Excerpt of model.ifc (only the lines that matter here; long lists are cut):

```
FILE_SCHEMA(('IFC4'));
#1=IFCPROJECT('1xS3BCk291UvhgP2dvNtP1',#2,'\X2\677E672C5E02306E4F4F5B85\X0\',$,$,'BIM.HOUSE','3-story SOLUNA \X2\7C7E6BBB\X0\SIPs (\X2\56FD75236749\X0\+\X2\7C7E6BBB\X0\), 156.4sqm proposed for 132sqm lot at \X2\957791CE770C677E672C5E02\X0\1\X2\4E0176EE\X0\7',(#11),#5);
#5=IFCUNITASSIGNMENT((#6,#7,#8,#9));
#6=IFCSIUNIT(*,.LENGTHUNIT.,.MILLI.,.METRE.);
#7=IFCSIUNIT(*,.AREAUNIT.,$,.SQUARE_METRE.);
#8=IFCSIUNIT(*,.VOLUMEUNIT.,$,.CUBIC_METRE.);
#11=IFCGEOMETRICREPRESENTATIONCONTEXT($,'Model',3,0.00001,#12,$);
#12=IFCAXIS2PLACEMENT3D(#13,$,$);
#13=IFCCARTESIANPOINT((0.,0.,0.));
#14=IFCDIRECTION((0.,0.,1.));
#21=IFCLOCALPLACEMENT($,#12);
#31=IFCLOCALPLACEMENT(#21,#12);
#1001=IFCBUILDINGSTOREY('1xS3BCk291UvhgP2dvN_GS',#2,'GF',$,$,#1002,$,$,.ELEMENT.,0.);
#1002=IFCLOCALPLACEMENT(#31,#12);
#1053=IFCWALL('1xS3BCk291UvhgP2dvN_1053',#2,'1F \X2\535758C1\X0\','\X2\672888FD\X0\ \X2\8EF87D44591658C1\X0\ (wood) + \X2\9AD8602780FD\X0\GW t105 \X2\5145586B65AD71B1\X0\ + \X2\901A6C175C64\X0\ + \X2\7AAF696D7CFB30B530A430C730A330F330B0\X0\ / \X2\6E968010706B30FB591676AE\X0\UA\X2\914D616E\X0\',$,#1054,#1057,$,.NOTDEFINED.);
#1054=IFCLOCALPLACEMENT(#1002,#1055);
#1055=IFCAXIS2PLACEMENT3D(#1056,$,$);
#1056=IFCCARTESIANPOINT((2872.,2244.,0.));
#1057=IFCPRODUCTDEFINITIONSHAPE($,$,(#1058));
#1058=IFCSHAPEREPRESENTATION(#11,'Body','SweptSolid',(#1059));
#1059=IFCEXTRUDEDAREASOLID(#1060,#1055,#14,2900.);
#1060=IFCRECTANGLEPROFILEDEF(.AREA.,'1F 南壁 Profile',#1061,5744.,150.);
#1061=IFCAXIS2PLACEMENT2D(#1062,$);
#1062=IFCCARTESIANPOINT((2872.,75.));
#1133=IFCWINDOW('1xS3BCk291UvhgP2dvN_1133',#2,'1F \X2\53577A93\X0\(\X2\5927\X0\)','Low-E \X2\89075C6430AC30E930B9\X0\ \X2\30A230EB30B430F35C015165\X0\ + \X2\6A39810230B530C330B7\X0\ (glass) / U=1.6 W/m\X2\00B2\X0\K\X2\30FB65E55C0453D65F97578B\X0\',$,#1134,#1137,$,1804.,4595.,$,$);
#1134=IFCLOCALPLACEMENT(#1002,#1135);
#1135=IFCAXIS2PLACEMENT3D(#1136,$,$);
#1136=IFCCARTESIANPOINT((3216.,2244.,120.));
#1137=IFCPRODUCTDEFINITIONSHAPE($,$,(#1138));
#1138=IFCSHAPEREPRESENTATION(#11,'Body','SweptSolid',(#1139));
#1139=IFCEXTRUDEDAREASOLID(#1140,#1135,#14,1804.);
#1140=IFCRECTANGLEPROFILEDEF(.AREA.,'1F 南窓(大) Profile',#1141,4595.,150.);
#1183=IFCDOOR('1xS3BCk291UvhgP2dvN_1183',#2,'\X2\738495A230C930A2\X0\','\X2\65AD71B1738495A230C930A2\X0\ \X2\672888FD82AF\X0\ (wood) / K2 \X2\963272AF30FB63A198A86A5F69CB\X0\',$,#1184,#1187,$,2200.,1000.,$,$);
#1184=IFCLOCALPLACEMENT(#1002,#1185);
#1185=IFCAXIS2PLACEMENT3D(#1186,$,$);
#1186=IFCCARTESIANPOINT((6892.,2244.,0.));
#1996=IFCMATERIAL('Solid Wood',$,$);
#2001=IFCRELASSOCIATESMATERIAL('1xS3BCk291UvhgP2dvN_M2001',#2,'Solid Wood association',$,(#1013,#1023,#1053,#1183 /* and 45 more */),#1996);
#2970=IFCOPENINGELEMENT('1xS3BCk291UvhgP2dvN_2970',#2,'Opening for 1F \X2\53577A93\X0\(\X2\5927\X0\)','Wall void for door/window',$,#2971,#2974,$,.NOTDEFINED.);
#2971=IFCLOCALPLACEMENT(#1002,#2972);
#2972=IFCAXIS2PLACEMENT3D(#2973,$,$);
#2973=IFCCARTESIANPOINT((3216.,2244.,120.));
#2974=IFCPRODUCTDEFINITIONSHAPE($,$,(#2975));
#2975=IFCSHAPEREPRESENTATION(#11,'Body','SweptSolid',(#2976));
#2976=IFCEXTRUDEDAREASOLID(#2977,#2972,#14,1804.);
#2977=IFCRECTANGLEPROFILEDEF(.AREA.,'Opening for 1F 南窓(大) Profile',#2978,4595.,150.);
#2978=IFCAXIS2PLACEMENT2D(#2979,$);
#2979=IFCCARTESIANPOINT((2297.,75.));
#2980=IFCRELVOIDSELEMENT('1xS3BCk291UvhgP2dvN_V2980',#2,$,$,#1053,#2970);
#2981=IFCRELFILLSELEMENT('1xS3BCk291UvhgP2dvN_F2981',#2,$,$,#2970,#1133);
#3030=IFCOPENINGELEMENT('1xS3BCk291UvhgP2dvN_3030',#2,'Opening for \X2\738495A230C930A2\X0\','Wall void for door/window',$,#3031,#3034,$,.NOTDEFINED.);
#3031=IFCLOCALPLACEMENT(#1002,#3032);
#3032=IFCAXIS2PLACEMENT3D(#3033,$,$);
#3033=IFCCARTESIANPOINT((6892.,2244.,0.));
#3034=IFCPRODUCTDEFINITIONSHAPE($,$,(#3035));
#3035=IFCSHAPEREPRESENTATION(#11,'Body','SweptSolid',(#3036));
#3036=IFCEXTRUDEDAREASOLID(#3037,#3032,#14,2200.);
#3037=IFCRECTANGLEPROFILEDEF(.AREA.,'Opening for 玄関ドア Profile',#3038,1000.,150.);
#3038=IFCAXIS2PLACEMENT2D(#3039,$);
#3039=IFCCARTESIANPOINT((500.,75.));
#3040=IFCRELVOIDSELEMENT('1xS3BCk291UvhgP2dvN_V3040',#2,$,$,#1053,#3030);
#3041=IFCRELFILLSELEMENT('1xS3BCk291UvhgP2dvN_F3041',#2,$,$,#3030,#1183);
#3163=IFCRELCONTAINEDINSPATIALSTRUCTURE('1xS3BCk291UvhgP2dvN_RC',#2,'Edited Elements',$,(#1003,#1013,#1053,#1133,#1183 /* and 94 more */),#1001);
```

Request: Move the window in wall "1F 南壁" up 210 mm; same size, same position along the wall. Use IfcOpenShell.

```python
import numpy as np
import ifcopenshell
import ifcopenshell.api.geometry
import ifcopenshell.util.placement
import ifcopenshell.util.unit

model = ifcopenshell.open("model.ifc")
unit_scale = ifcopenshell.util.unit.calculate_unit_scale(model)

window = model.by_guid("1xS3BCk291UvhgP2dvN_1133")
opening = window.FillsVoids[0].RelatingOpeningElement
dz = 210.0

shift = np.array([0.0, 0.0, dz])
# The window is not placed relative to its opening, so move both.
for product in (opening, window):
    matrix = ifcopenshell.util.placement.get_local_placement(product.ObjectPlacement)
    matrix[:3, 3] += shift
    ifcopenshell.api.geometry.edit_object_placement(model, product=product, matrix=matrix, is_si=False)

print(f"moved by {dz * unit_scale:+.3f} m")

model.write("model_v2.ifc")
```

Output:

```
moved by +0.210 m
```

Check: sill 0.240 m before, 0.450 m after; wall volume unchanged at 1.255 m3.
